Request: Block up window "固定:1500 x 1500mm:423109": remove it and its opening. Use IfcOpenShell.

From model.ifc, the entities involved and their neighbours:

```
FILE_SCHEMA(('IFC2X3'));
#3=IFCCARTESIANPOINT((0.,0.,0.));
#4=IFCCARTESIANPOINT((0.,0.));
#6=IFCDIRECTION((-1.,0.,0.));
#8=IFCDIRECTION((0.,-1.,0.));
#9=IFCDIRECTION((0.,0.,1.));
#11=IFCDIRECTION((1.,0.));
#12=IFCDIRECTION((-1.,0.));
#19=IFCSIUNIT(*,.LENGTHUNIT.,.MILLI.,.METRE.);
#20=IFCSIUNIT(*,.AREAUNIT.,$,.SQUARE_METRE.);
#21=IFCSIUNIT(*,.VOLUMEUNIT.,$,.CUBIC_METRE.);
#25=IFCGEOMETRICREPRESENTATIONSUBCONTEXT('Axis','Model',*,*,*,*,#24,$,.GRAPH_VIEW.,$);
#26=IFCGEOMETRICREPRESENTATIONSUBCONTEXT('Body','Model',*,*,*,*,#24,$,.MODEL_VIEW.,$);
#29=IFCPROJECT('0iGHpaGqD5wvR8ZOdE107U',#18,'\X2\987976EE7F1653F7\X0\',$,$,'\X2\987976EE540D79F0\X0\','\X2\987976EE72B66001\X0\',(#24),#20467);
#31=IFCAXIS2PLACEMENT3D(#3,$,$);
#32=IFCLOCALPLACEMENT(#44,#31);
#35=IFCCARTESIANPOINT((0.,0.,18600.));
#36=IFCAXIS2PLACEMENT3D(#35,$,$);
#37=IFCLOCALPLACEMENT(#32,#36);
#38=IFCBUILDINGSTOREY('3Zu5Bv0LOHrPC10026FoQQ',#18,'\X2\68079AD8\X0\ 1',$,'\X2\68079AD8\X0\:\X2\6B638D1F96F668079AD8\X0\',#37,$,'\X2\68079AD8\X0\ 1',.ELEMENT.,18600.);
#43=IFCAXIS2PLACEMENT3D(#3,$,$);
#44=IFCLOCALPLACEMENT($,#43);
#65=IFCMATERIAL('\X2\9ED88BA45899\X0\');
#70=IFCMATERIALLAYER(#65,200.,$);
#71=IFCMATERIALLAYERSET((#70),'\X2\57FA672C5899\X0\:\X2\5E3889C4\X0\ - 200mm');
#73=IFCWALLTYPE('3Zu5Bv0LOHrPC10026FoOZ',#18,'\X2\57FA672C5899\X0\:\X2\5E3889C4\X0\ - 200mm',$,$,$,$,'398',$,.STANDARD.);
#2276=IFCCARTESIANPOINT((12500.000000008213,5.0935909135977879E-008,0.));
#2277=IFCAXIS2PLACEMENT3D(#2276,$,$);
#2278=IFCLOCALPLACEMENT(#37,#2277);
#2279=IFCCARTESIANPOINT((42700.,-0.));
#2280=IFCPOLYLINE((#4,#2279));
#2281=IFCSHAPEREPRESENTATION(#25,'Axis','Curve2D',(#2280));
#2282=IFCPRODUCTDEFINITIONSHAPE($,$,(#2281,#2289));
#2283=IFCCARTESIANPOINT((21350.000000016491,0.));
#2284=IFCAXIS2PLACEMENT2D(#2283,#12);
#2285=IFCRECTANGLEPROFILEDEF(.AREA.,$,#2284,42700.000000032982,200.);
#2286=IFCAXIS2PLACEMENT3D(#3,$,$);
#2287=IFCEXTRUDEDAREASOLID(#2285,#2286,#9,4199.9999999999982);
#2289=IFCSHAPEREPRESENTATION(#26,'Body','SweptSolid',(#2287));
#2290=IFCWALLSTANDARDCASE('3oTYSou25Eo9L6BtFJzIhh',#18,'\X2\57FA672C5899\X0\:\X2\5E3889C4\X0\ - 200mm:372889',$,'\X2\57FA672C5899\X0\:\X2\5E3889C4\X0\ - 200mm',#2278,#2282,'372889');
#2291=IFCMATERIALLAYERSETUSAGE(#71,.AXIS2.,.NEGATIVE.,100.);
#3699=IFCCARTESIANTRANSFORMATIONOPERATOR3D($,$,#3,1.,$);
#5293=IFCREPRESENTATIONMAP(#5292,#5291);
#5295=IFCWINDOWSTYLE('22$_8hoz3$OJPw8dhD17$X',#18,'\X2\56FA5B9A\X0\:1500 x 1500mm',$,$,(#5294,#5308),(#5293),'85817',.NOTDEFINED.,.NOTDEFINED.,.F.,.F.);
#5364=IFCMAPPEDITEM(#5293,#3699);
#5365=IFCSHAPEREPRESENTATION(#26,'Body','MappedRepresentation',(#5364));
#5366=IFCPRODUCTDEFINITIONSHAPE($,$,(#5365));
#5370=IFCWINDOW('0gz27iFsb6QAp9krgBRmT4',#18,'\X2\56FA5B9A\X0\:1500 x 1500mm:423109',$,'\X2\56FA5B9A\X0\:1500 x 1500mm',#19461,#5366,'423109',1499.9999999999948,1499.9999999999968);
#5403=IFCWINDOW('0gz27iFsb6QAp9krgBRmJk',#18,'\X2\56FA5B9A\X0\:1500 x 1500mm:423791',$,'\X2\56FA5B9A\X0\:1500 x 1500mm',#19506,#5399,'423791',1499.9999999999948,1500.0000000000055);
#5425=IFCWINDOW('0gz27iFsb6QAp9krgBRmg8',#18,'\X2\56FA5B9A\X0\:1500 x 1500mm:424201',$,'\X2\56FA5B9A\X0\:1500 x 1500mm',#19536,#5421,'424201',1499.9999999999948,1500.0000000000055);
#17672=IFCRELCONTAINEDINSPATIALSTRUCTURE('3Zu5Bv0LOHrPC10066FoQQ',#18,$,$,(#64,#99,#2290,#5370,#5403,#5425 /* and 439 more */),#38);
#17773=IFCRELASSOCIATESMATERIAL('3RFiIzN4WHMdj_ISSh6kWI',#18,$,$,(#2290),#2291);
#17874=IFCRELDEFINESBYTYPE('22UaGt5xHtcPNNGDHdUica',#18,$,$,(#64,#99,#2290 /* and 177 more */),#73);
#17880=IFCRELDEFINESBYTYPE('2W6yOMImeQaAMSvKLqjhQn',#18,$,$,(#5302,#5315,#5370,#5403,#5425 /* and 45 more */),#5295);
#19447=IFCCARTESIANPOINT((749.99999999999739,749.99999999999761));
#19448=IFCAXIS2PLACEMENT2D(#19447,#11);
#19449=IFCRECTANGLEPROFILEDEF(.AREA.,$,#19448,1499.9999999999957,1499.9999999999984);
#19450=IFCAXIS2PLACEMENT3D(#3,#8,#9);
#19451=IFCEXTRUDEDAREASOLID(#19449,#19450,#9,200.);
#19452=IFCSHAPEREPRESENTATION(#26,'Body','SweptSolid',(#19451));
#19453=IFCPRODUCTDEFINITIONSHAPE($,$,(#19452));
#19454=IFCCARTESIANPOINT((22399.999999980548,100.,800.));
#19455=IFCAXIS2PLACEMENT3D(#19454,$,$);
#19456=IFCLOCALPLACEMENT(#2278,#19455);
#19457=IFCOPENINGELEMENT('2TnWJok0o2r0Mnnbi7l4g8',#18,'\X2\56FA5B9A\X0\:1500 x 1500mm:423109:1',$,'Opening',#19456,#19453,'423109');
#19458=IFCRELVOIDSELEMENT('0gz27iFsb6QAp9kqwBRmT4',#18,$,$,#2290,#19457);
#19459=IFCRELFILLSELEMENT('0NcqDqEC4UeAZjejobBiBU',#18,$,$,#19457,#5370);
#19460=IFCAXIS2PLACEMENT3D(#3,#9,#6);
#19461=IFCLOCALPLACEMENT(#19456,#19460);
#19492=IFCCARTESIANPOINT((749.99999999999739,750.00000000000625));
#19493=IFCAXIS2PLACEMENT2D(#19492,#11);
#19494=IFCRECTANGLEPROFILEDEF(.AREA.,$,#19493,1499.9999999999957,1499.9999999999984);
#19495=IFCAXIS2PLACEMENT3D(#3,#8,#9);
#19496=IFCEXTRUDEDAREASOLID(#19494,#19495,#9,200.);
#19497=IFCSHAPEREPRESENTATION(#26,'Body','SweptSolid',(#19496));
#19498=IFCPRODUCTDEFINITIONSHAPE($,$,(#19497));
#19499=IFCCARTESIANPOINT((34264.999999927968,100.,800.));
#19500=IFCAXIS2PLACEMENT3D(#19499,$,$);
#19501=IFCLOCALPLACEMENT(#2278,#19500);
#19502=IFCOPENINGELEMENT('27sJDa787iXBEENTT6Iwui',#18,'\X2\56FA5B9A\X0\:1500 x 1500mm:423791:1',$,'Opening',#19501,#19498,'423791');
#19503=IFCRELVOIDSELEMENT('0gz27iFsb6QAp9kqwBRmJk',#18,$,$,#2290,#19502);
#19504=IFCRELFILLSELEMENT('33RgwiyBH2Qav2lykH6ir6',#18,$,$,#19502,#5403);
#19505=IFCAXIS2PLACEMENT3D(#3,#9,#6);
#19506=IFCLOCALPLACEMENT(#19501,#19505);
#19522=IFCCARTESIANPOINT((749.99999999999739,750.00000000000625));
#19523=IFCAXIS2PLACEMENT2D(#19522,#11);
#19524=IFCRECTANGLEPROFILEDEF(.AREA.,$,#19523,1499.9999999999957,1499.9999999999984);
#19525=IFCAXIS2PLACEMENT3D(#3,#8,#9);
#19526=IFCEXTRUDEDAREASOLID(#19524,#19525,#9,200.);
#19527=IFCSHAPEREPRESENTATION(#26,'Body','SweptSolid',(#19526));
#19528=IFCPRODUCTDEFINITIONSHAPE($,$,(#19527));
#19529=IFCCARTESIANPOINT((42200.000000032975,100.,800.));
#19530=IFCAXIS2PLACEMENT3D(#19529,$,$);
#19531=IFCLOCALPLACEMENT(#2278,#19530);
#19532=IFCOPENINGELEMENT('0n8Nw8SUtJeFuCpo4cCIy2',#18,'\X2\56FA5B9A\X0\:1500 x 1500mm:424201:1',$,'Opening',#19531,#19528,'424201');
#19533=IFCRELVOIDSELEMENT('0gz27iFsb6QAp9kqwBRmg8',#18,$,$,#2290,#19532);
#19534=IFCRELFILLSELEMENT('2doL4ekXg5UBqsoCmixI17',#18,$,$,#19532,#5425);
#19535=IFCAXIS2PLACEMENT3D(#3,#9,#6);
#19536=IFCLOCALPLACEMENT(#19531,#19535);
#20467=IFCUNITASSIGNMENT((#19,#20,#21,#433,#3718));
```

```python
import ifcopenshell
import ifcopenshell.api.feature
import ifcopenshell.api.root
import ifcopenshell.geom
import ifcopenshell.util.shape

model = ifcopenshell.open("model.ifc")
settings = ifcopenshell.geom.settings()


def volume(element):
    """Net volume in cubic metres, openings subtracted."""
    shape = ifcopenshell.geom.create_shape(settings, element)
    return ifcopenshell.util.shape.get_volume(shape.geometry)


window = model.by_id(5370)
opening = window.FillsVoids[0].RelatingOpeningElement
wall = opening.VoidsElements[0].RelatingBuildingElement
before = volume(wall)

ifcopenshell.api.root.remove_product(model, product=window)
ifcopenshell.api.feature.remove_feature(model, feature=opening)

after = volume(wall)

print(f"wall volume {before:.3f} -> {after:.3f} m3")

model.write("model_edited.ifc")
```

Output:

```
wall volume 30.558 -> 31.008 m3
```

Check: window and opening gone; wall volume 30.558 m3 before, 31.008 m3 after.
